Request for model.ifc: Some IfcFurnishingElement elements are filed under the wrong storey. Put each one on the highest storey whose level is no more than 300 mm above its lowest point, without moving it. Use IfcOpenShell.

First a look at what the model holds.

```python
import ifcopenshell
import ifcopenshell.util.element
import ifcopenshell.util.placement

model = ifcopenshell.open("model.ifc")
print(model.schema)
for storey in model.by_type("IfcBuildingStorey"):
    level = ifcopenshell.util.placement.get_storey_elevation(storey)
    count = sum(e.is_a("IfcFurnishingElement") for e in ifcopenshell.util.element.get_contained(storey))
    print(storey.id(), storey.Name, round(level, 3), count, sep=" | ")
```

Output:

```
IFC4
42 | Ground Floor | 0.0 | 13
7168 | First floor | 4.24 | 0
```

```python
import ifcopenshell
import ifcopenshell.api.spatial
import ifcopenshell.geom
import ifcopenshell.util.element
import ifcopenshell.util.placement
import ifcopenshell.util.shape
import ifcopenshell.util.unit

model = ifcopenshell.open("model.ifc")
unit_scale = ifcopenshell.util.unit.calculate_unit_scale(model)
settings = ifcopenshell.geom.settings()

levels = sorted(
    ((ifcopenshell.util.placement.get_storey_elevation(s) * unit_scale, s) for s in model.by_type("IfcBuildingStorey")),
    key=lambda pair: pair[0],
)

for e in model.by_type("IfcFurnishingElement"):
    current = e.ContainedInStructure[0].RelatingStructure if e.ContainedInStructure else None
    if current is None or not current.is_a("IfcBuildingStorey"):
        continue
    shape = ifcopenshell.geom.create_shape(settings, e)
    bottom = ifcopenshell.util.shape.get_shape_bottom_elevation(shape, shape.geometry)
    below = [s for level, s in levels if level <= bottom + 0.3]
    storey = below[-1] if below else levels[0][1]
    if storey != current:
        # assign_container keeps the world position.
        ifcopenshell.api.spatial.assign_container(model, products=[e], relating_structure=storey)
        print(e.id(), current.Name, "->", storey.Name)

model.write("model_v2.ifc")
```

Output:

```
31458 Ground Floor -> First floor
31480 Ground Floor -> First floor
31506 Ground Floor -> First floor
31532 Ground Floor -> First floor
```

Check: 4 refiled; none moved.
